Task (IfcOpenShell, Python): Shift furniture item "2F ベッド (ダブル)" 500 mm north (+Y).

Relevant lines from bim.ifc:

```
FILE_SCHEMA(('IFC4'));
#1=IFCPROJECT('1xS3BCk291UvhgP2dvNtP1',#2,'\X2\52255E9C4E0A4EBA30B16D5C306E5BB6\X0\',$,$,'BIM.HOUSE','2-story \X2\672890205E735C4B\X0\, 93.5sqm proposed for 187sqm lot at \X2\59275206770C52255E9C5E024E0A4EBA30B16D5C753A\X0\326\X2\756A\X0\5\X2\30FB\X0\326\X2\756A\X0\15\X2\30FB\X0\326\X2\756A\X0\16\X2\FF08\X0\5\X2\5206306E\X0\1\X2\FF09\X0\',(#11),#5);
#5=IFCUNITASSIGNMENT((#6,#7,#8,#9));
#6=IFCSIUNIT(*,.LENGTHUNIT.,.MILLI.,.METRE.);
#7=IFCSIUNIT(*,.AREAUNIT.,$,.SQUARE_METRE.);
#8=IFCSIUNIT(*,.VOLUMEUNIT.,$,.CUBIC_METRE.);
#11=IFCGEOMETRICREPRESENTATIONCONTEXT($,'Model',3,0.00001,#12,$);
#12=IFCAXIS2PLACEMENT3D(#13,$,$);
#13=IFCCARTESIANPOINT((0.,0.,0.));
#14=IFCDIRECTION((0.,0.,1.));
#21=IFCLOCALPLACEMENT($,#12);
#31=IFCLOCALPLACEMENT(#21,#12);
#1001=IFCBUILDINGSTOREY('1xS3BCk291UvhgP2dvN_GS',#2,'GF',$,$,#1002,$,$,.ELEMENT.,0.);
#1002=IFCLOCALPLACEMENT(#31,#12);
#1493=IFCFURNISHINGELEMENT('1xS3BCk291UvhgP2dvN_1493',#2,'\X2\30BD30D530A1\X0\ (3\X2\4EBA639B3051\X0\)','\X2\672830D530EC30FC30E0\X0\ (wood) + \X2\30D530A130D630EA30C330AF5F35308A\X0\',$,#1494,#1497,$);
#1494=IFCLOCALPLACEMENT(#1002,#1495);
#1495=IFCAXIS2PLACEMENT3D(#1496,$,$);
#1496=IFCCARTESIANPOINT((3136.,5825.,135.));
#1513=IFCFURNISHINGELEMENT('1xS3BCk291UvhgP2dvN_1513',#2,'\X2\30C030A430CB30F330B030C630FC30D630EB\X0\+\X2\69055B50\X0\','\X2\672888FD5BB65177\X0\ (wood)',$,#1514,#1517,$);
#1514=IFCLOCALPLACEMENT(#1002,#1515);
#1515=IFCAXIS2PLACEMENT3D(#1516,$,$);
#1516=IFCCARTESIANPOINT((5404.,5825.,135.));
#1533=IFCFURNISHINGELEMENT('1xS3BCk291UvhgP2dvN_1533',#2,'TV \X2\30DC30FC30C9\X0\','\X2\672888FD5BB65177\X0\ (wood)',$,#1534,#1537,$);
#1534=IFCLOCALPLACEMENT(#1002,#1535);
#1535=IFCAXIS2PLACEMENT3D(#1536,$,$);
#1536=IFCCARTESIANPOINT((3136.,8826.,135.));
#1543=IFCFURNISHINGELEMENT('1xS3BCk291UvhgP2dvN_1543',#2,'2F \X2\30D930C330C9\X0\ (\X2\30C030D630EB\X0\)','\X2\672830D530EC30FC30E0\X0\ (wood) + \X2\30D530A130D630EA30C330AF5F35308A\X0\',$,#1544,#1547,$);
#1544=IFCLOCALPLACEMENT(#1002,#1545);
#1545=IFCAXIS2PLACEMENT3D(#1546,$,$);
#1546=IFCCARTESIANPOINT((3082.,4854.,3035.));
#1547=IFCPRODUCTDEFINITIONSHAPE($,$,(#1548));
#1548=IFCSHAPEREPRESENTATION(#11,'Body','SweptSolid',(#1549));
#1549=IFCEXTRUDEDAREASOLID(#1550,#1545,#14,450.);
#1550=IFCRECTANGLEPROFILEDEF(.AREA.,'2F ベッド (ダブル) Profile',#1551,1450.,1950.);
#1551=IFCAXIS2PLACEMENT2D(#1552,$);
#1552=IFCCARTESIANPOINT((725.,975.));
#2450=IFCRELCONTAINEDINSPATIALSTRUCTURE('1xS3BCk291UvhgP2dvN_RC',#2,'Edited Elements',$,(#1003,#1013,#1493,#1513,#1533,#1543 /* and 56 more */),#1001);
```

```python
import ifcopenshell
import ifcopenshell.api.geometry
import ifcopenshell.util.placement
import ifcopenshell.util.unit

model = ifcopenshell.open("bim.ifc")
unit_scale = ifcopenshell.util.unit.calculate_unit_scale(model)

item = model.by_guid("1xS3BCk291UvhgP2dvN_1543")
matrix = ifcopenshell.util.placement.get_local_placement(item.ObjectPlacement)
matrix[1, 3] += 0.5 / unit_scale
ifcopenshell.api.geometry.edit_object_placement(model, product=item, matrix=matrix, is_si=False)

print(ifcopenshell.util.placement.get_local_placement(item.ObjectPlacement).round(3) + 0.0)

model.write("bim_edited.ifc")
```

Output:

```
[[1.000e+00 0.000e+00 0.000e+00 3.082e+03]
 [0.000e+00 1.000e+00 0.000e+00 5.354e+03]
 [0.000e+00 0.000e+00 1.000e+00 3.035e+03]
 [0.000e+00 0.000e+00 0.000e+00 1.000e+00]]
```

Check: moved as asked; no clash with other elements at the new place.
